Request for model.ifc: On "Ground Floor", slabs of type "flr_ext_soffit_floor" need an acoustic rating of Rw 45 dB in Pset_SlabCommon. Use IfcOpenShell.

First a look at what the model holds.

```python
import ifcopenshell
import ifcopenshell.util.element

model = ifcopenshell.open("model.ifc")
print(model.schema)
storey = next(s for s in model.by_type("IfcBuildingStorey") if s.Name == "Ground Floor")
slabs = [e for e in ifcopenshell.util.element.get_decomposition(storey) if e.is_a("IfcSlab")]
seen = {}
for e in slabs:
    element_type = ifcopenshell.util.element.get_type(e)
    key = (element_type.Name if element_type != e and element_type else None, ifcopenshell.util.element.get_pset(e, "Pset_SlabCommon", "AcousticRating"))
    seen[key] = seen.get(key, 0) + 1
for (name, value), count in sorted(seen.items(), key=str):
    print(count, "x", name, "|", value)
```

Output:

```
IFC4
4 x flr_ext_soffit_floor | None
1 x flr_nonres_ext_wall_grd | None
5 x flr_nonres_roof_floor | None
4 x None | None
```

```python
import ifcopenshell
import ifcopenshell.api.pset
import ifcopenshell.util.element

model = ifcopenshell.open("model.ifc")

storey = next(s for s in model.by_type("IfcBuildingStorey") if s.Name == "Ground Floor")
slabs = [e for e in ifcopenshell.util.element.get_decomposition(storey) if e.is_a("IfcSlab")]

count = 0
for e in slabs:
    element_type = ifcopenshell.util.element.get_type(e)
    if element_type in (None, e) or element_type.Name != "flr_ext_soffit_floor":
        continue
    # add_pset returns the element's existing set when there is one.
    pset = ifcopenshell.api.pset.add_pset(model, product=e, name="Pset_SlabCommon")
    ifcopenshell.api.pset.edit_pset(model, pset=pset, properties={"AcousticRating": "Rw 45 dB"})
    count += 1

print(count, "slabs updated")

model.write("model_rev.ifc")
```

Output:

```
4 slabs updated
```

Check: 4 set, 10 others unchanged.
